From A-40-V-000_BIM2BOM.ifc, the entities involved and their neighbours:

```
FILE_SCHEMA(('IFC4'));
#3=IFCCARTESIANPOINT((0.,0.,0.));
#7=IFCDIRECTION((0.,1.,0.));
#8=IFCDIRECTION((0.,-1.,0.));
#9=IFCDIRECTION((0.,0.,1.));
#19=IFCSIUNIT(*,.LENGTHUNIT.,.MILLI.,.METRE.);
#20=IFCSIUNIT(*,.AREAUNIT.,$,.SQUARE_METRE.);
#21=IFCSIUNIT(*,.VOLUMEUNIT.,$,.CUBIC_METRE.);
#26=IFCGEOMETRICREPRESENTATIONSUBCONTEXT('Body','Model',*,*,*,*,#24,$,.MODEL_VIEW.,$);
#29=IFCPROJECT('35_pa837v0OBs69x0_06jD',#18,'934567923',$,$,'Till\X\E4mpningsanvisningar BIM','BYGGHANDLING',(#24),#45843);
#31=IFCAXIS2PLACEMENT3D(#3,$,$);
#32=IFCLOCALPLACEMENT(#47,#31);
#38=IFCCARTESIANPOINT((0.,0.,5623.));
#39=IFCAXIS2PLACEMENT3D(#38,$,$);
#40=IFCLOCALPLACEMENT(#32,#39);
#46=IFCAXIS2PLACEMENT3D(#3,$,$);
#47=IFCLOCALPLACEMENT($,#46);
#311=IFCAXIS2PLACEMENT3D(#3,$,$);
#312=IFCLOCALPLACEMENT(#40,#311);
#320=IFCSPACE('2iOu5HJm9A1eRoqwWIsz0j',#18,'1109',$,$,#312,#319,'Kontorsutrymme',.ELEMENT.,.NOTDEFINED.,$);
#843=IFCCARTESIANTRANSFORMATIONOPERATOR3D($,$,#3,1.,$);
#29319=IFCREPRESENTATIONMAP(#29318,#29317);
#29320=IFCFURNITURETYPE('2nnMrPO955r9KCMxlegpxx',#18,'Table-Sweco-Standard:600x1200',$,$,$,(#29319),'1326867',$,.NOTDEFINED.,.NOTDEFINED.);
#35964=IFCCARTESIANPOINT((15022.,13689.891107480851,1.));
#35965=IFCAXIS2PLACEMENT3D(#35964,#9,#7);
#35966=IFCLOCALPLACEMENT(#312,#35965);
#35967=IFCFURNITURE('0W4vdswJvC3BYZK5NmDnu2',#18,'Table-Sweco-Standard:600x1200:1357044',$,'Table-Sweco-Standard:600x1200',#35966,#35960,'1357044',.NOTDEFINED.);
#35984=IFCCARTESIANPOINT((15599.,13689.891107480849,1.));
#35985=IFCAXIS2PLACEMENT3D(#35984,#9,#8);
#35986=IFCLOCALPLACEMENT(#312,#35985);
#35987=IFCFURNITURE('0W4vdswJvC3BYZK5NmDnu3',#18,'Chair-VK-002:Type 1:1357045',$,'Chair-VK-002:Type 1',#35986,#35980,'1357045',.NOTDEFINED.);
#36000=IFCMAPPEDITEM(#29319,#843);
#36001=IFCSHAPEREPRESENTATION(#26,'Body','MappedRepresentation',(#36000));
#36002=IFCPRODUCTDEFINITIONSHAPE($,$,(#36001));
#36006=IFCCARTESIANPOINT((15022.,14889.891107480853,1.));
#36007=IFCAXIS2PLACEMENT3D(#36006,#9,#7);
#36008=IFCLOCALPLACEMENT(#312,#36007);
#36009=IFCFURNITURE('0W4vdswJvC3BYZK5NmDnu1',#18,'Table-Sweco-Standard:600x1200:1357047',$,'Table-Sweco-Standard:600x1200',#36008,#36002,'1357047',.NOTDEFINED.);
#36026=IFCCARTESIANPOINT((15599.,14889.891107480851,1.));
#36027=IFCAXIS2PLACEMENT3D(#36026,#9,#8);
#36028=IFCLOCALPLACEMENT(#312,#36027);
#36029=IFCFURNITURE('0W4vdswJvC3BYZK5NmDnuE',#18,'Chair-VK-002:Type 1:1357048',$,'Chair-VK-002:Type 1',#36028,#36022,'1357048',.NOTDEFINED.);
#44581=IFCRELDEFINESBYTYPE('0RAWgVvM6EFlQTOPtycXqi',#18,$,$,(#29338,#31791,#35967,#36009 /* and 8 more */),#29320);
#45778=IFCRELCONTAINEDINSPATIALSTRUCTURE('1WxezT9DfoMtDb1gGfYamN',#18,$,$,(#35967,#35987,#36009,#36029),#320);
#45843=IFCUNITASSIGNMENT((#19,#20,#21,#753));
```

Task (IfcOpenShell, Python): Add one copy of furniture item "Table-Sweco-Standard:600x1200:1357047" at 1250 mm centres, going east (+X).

```python
import numpy as np
import ifcopenshell
import ifcopenshell.api.geometry
import ifcopenshell.api.root
import ifcopenshell.util.element
import ifcopenshell.util.placement
import ifcopenshell.util.unit

model = ifcopenshell.open("A-40-V-000_BIM2BOM.ifc")
unit_scale = ifcopenshell.util.unit.calculate_unit_scale(model)


def reuse_history(source, copy):
    """copy_class also copies each property set's owner history, people and application; keep the originals."""
    for rel in copy.IsDefinedBy:
        if rel.is_a("IfcRelDefinesByProperties") and (history := rel.RelatingPropertyDefinition.OwnerHistory):
            rel.RelatingPropertyDefinition.OwnerHistory = source.OwnerHistory
            ifcopenshell.util.element.remove_deep2(model, history)


source = model.by_guid("0W4vdswJvC3BYZK5NmDnu1")
base = ifcopenshell.util.placement.get_local_placement(source.ObjectPlacement)
step = np.array([1.0, 0.0, 0.0]) * 1.25 / unit_scale

for i in range(1, 2):
    copy = ifcopenshell.api.root.copy_class(model, product=source)
    copy.Representation = ifcopenshell.util.element.copy_deep(
        model, source.Representation, exclude=["IfcGeometricRepresentationContext", "IfcRepresentationMap"]
    )
    copy.Name = "Table-Sweco-Standard:600x1200"
    copy.Tag = None
    reuse_history(source, copy)
    matrix = base.copy()
    matrix[:3, 3] += i * step
    print("added at", matrix[:3, 3].round(3) + 0.0)
    ifcopenshell.api.geometry.edit_object_placement(model, product=copy, matrix=matrix, is_si=False)

model.write("A-40-V-000_BIM2BOM_v2.ifc")
```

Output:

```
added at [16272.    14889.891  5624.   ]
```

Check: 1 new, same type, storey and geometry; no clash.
